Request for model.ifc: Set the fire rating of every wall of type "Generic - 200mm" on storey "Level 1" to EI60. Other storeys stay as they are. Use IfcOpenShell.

First a look at what the model holds.

```python
import ifcopenshell
import ifcopenshell.util.element

model = ifcopenshell.open("model.ifc")
print(model.schema)
storey = next(s for s in model.by_type("IfcBuildingStorey") if s.Name == "Level 1")
walls = [e for e in ifcopenshell.util.element.get_decomposition(storey) if e.is_a("IfcWall")]
seen = {}
for e in walls:
    element_type = ifcopenshell.util.element.get_type(e)
    key = (element_type.Name if element_type != e and element_type else None, ifcopenshell.util.element.get_pset(e, "Pset_WallCommon", "FireRating"))
    seen[key] = seen.get(key, 0) + 1
for (name, value), count in sorted(seen.items(), key=str):
    print(count, "x", name, "|", value)
```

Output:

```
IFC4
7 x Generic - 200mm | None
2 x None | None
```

```python
import ifcopenshell
import ifcopenshell.api.pset
import ifcopenshell.util.element

model = ifcopenshell.open("model.ifc")

storey = next(s for s in model.by_type("IfcBuildingStorey") if s.Name == "Level 1")
walls = [e for e in ifcopenshell.util.element.get_decomposition(storey) if e.is_a("IfcWall")]

count = 0
for e in walls:
    element_type = ifcopenshell.util.element.get_type(e)
    if element_type in (None, e) or element_type.Name != "Generic - 200mm":
        continue
    # add_pset returns the element's existing set when there is one.
    pset = ifcopenshell.api.pset.add_pset(model, product=e, name="Pset_WallCommon")
    ifcopenshell.api.pset.edit_pset(model, pset=pset, properties={"FireRating": "EI60"})
    count += 1

print(count, "walls updated")

model.write("model_v2.ifc")
```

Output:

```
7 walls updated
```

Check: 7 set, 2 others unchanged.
